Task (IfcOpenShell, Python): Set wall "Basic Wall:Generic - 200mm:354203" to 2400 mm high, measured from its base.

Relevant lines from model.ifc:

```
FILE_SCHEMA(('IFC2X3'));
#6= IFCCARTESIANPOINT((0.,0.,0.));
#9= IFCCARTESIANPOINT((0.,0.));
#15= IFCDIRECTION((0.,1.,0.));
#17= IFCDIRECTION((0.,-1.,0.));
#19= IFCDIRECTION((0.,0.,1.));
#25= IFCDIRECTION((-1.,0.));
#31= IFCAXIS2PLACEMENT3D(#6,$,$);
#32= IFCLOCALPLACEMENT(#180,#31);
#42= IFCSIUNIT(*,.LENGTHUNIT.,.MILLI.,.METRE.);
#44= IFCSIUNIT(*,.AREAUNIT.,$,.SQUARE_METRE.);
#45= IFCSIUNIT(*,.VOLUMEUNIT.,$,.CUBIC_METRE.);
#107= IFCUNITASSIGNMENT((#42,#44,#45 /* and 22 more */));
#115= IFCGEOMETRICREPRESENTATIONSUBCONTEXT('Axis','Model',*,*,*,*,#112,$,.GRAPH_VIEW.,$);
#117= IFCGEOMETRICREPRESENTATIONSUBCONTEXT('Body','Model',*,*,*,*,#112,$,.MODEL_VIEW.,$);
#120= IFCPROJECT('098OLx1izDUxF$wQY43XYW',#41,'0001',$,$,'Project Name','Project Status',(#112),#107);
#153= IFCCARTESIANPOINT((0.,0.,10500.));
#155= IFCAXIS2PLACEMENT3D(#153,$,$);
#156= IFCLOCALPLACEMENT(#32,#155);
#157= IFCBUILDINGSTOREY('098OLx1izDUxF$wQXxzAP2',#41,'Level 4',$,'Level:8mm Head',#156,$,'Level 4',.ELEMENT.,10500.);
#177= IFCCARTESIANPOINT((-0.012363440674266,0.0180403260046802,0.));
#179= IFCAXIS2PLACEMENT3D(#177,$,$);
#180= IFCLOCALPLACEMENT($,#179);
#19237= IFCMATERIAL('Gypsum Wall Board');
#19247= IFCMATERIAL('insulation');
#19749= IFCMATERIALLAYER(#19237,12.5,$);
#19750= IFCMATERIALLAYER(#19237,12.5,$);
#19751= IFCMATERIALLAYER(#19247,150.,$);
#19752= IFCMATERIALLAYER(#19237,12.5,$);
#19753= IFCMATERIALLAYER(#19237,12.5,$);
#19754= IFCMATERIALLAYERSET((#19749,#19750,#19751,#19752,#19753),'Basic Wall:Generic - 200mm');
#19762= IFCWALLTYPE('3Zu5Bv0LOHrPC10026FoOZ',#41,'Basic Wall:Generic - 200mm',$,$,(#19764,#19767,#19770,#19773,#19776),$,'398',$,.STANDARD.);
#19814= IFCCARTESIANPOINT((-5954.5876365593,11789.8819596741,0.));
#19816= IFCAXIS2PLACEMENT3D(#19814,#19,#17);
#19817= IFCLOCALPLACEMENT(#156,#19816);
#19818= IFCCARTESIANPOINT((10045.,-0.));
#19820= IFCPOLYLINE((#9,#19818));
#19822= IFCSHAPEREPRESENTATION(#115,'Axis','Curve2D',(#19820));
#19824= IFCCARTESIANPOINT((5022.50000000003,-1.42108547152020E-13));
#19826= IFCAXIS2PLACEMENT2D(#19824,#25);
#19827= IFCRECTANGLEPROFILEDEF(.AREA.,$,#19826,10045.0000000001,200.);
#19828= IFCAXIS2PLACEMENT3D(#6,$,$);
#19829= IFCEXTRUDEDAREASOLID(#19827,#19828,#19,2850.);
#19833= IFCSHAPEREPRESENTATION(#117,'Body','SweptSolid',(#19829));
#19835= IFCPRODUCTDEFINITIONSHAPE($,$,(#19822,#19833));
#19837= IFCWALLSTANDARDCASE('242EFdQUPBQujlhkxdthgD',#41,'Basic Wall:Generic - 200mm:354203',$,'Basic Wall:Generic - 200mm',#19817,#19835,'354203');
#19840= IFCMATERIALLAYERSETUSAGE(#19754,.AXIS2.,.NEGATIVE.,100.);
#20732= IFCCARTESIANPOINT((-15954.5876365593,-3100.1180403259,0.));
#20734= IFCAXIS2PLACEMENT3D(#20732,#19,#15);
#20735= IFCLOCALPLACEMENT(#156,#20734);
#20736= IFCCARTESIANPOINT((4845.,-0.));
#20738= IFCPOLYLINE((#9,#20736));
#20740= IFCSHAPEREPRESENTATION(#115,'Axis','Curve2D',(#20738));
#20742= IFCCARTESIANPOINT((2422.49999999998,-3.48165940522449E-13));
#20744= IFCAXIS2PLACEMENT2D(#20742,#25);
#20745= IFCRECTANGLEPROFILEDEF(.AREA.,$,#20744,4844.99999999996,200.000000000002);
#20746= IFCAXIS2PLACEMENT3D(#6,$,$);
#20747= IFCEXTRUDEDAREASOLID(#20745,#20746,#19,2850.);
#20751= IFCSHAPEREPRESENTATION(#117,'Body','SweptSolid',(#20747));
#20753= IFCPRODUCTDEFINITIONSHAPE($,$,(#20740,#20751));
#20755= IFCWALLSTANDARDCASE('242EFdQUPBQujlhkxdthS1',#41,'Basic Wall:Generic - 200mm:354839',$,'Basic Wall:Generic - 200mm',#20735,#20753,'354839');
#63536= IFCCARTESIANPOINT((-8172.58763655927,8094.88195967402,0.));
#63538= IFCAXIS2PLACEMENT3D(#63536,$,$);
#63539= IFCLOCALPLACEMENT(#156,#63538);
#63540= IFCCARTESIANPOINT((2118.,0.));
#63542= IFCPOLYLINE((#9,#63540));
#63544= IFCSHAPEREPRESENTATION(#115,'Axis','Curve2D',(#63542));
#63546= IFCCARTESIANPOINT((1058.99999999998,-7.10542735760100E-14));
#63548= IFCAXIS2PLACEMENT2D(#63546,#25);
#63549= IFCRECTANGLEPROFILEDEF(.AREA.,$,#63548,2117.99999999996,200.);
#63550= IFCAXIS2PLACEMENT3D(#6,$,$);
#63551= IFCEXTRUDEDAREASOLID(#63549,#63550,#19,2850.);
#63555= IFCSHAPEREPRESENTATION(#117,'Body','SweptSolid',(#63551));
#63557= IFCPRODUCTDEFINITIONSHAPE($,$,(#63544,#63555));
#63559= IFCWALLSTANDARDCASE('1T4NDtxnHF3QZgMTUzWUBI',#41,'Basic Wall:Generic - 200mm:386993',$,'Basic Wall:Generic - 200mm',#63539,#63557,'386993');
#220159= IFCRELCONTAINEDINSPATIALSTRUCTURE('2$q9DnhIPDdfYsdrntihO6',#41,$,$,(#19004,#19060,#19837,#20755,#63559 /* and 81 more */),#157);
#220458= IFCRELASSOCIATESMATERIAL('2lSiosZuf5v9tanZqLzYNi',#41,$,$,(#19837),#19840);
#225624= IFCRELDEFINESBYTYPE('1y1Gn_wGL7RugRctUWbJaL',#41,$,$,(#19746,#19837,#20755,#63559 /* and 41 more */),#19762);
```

```python
import ifcopenshell
import ifcopenshell.geom
import ifcopenshell.util.representation
import ifcopenshell.util.shape
import ifcopenshell.util.unit

model = ifcopenshell.open("model.ifc")
unit_scale = ifcopenshell.util.unit.calculate_unit_scale(model)
settings = ifcopenshell.geom.settings()


def volume(element):
    """Net volume in cubic metres, openings subtracted."""
    shape = ifcopenshell.geom.create_shape(settings, element)
    return ifcopenshell.util.shape.get_volume(shape.geometry)


wall = model.by_guid("242EFdQUPBQujlhkxdthgD")
before = volume(wall)

body = ifcopenshell.util.representation.get_representation(wall, "Model", "Body")
solid = body.Items[0]
old_height = solid.Depth
solid.Depth = 2.4 / unit_scale
after = volume(wall)

print(f"height {old_height:g} -> {solid.Depth:g}, volume {before:.3f} -> {after:.3f} m3")

model.write("model_rev.ifc")
```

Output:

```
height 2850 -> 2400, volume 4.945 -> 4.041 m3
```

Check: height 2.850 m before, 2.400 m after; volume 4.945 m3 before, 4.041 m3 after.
